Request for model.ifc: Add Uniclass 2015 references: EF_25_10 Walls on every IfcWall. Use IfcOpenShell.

First a look at what the model holds.

```python
import ifcopenshell

model = ifcopenshell.open("model.ifc")
print(model.schema)
print("classifications:", [c.Name for c in model.by_type("IfcClassification")])
for ifc_class in ("IfcDoor", "IfcRoof", "IfcStair", "IfcWall", "IfcWindow"):
    print(ifc_class, len(model.by_type(ifc_class)))
```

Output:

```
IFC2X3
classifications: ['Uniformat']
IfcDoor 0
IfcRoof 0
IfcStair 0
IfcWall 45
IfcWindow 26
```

```python
import ifcopenshell
import ifcopenshell.api.classification

model = ifcopenshell.open("model.ifc")

# IFC2X3 requires Source and Edition and has no link from the project to the system.
system = model.create_entity("IfcClassification", Source="NBS", Edition="2015", Name="Uniclass 2015")

codes = {
    "IfcWall": ("EF_25_10", "Walls"),
}
for ifc_class, (code, name) in codes.items():
    products = model.by_type(ifc_class)
    ifcopenshell.api.classification.add_reference(
        model, products=products, classification=system, identification=code, name=name
    )
    print(code, len(products))

model.write("model_v2.ifc")
```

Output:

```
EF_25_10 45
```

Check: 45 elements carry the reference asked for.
